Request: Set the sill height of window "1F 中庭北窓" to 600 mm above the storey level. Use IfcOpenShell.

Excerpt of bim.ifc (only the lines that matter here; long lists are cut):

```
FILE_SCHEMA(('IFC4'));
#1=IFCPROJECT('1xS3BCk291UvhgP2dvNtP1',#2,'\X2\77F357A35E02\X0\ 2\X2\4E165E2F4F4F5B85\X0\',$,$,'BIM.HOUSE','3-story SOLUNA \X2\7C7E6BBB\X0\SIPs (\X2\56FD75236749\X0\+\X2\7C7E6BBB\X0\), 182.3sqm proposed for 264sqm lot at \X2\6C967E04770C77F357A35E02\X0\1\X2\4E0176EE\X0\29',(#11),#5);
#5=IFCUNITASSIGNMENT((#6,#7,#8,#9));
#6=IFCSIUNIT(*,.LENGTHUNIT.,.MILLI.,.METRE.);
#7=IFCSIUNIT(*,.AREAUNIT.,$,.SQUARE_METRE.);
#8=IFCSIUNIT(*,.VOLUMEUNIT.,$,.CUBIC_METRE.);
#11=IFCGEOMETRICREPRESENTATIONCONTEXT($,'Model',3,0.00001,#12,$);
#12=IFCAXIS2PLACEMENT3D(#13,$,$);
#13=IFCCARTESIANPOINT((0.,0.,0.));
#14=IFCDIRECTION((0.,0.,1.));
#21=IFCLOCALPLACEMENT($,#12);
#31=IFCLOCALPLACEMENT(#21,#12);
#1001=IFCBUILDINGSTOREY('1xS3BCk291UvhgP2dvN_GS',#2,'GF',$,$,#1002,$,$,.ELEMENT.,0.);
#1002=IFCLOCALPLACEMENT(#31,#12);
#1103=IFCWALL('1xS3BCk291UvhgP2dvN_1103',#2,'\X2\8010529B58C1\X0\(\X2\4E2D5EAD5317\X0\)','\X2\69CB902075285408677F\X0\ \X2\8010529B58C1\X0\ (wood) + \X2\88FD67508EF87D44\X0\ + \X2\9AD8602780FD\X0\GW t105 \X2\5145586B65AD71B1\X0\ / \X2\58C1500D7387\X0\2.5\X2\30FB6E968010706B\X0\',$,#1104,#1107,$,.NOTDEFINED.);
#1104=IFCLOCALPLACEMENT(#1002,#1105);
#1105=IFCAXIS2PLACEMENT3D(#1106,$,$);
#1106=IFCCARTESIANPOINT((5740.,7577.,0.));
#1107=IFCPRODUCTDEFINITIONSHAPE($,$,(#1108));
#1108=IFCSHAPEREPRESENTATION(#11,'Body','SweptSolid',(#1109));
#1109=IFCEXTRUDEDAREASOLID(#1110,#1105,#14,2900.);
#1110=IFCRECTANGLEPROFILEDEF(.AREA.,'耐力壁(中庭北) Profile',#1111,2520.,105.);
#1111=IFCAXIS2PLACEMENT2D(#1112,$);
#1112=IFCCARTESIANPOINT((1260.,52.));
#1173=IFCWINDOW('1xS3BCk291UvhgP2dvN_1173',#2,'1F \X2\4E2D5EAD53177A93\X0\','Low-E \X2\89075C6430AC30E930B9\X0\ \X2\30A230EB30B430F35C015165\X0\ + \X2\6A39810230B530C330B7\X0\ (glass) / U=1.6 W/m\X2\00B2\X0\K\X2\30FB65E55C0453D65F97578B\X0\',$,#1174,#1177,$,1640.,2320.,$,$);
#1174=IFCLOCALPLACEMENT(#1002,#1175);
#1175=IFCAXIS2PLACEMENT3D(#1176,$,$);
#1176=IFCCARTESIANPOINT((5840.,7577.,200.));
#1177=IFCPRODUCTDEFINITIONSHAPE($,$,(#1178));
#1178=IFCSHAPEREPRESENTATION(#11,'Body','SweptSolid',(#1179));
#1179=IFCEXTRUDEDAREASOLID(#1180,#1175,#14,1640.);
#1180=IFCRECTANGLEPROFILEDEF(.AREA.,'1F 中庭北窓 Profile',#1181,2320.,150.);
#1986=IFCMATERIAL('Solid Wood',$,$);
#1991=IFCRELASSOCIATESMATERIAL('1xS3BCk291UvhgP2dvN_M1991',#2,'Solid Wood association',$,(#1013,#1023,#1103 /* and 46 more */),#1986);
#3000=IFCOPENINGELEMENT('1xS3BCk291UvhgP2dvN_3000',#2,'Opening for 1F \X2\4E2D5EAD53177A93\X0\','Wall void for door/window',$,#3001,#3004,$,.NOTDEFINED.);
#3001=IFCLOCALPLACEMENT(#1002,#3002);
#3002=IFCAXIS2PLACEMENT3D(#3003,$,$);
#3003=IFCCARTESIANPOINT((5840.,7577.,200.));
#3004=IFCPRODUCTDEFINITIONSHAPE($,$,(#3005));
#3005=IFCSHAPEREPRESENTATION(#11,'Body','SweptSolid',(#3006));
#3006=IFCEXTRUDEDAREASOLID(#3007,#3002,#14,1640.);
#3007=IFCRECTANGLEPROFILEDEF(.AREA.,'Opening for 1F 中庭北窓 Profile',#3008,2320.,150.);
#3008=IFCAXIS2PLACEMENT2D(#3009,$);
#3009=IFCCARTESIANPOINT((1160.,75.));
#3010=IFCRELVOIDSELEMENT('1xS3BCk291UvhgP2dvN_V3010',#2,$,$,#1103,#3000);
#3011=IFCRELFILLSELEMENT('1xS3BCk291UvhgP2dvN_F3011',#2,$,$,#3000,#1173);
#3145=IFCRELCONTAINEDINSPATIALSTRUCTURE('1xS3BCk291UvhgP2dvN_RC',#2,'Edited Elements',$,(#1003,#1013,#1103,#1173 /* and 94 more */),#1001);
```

```python
import numpy as np
import ifcopenshell
import ifcopenshell.api.geometry
import ifcopenshell.geom
import ifcopenshell.util.element
import ifcopenshell.util.placement
import ifcopenshell.util.shape
import ifcopenshell.util.unit

model = ifcopenshell.open("bim.ifc")
unit_scale = ifcopenshell.util.unit.calculate_unit_scale(model)

window = model.by_guid("1xS3BCk291UvhgP2dvN_1173")
opening = window.FillsVoids[0].RelatingOpeningElement
storey = ifcopenshell.util.element.get_container(window, ifc_class="IfcBuildingStorey")
level = ifcopenshell.util.placement.get_local_placement(storey.ObjectPlacement)[2, 3]

# The opening's origin need not be at the sill, so measure its lowest point.
shape = ifcopenshell.geom.create_shape(ifcopenshell.geom.settings(), opening)
bottom = ifcopenshell.util.shape.get_shape_bottom_elevation(shape, shape.geometry) / unit_scale
dz = level + 0.6 / unit_scale - bottom

shift = np.array([0.0, 0.0, dz])
# The window is not placed relative to its opening, so move both.
for product in (opening, window):
    matrix = ifcopenshell.util.placement.get_local_placement(product.ObjectPlacement)
    matrix[:3, 3] += shift
    ifcopenshell.api.geometry.edit_object_placement(model, product=product, matrix=matrix, is_si=False)

print(f"moved by {dz * unit_scale:+.3f} m")

model.write("bim_rev.ifc")
```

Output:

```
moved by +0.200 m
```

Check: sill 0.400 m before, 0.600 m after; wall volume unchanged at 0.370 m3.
